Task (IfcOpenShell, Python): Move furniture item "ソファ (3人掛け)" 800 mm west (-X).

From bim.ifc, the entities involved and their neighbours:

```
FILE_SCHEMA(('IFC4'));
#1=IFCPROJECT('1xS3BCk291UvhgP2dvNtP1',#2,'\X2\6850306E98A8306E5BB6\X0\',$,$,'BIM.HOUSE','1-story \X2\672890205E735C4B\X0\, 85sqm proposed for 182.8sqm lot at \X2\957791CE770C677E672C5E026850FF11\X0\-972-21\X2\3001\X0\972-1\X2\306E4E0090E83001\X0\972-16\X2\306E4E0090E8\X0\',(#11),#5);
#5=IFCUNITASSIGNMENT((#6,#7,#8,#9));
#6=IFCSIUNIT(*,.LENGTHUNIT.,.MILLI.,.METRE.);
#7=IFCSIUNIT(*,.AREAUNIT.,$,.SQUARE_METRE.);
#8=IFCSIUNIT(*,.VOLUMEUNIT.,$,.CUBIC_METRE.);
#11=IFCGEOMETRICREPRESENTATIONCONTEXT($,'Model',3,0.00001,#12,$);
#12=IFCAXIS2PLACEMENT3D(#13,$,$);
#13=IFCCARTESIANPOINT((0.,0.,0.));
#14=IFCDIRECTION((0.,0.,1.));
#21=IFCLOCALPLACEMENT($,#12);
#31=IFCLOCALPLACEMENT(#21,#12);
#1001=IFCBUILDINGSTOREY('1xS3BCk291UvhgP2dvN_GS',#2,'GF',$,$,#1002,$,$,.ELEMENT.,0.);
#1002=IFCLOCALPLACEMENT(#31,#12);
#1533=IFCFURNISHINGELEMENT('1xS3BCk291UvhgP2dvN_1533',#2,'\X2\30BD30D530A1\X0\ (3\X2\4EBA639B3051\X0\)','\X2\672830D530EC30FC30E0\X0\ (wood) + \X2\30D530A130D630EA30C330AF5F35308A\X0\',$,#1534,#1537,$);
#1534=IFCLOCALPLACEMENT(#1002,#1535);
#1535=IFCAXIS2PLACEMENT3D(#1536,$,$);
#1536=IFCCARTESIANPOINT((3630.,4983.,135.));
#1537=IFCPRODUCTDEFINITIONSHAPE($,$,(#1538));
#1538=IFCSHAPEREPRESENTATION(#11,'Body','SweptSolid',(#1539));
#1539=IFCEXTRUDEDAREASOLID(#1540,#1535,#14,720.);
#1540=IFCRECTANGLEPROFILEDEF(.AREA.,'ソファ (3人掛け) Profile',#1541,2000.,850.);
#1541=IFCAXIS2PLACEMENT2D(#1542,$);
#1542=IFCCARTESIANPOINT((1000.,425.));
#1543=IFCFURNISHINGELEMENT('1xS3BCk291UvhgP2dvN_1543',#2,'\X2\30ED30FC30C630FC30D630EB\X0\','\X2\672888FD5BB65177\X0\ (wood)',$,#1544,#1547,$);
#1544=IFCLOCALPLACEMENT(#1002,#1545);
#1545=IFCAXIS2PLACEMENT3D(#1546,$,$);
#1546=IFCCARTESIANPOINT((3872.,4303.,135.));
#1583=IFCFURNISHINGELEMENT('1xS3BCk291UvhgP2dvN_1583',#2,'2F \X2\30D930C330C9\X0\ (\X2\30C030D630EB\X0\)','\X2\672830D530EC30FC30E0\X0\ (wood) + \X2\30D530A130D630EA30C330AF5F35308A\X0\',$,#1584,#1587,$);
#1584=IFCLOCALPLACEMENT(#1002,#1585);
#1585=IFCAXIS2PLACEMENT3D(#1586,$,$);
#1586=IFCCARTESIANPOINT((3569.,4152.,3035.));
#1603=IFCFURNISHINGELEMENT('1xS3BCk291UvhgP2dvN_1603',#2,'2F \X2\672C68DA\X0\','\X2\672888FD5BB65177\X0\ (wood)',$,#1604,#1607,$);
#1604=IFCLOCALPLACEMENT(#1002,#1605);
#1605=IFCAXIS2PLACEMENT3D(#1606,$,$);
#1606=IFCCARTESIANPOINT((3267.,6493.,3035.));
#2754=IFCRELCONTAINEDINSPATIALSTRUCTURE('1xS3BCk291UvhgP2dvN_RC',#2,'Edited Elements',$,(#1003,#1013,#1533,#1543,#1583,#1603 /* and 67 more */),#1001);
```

```python
import ifcopenshell
import ifcopenshell.api.geometry
import ifcopenshell.util.placement

model = ifcopenshell.open("bim.ifc")

item = model.by_id(1533)
matrix = ifcopenshell.util.placement.get_local_placement(item.ObjectPlacement)
matrix[0, 3] -= 800.0
ifcopenshell.api.geometry.edit_object_placement(model, product=item, matrix=matrix, is_si=False)

print(ifcopenshell.util.placement.get_local_placement(item.ObjectPlacement).round(3) + 0.0)

model.write("bim_rev.ifc")
```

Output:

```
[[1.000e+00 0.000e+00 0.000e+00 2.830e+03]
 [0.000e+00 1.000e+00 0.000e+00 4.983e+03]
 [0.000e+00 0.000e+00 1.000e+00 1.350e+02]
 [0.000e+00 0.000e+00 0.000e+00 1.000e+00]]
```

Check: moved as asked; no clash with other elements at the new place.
